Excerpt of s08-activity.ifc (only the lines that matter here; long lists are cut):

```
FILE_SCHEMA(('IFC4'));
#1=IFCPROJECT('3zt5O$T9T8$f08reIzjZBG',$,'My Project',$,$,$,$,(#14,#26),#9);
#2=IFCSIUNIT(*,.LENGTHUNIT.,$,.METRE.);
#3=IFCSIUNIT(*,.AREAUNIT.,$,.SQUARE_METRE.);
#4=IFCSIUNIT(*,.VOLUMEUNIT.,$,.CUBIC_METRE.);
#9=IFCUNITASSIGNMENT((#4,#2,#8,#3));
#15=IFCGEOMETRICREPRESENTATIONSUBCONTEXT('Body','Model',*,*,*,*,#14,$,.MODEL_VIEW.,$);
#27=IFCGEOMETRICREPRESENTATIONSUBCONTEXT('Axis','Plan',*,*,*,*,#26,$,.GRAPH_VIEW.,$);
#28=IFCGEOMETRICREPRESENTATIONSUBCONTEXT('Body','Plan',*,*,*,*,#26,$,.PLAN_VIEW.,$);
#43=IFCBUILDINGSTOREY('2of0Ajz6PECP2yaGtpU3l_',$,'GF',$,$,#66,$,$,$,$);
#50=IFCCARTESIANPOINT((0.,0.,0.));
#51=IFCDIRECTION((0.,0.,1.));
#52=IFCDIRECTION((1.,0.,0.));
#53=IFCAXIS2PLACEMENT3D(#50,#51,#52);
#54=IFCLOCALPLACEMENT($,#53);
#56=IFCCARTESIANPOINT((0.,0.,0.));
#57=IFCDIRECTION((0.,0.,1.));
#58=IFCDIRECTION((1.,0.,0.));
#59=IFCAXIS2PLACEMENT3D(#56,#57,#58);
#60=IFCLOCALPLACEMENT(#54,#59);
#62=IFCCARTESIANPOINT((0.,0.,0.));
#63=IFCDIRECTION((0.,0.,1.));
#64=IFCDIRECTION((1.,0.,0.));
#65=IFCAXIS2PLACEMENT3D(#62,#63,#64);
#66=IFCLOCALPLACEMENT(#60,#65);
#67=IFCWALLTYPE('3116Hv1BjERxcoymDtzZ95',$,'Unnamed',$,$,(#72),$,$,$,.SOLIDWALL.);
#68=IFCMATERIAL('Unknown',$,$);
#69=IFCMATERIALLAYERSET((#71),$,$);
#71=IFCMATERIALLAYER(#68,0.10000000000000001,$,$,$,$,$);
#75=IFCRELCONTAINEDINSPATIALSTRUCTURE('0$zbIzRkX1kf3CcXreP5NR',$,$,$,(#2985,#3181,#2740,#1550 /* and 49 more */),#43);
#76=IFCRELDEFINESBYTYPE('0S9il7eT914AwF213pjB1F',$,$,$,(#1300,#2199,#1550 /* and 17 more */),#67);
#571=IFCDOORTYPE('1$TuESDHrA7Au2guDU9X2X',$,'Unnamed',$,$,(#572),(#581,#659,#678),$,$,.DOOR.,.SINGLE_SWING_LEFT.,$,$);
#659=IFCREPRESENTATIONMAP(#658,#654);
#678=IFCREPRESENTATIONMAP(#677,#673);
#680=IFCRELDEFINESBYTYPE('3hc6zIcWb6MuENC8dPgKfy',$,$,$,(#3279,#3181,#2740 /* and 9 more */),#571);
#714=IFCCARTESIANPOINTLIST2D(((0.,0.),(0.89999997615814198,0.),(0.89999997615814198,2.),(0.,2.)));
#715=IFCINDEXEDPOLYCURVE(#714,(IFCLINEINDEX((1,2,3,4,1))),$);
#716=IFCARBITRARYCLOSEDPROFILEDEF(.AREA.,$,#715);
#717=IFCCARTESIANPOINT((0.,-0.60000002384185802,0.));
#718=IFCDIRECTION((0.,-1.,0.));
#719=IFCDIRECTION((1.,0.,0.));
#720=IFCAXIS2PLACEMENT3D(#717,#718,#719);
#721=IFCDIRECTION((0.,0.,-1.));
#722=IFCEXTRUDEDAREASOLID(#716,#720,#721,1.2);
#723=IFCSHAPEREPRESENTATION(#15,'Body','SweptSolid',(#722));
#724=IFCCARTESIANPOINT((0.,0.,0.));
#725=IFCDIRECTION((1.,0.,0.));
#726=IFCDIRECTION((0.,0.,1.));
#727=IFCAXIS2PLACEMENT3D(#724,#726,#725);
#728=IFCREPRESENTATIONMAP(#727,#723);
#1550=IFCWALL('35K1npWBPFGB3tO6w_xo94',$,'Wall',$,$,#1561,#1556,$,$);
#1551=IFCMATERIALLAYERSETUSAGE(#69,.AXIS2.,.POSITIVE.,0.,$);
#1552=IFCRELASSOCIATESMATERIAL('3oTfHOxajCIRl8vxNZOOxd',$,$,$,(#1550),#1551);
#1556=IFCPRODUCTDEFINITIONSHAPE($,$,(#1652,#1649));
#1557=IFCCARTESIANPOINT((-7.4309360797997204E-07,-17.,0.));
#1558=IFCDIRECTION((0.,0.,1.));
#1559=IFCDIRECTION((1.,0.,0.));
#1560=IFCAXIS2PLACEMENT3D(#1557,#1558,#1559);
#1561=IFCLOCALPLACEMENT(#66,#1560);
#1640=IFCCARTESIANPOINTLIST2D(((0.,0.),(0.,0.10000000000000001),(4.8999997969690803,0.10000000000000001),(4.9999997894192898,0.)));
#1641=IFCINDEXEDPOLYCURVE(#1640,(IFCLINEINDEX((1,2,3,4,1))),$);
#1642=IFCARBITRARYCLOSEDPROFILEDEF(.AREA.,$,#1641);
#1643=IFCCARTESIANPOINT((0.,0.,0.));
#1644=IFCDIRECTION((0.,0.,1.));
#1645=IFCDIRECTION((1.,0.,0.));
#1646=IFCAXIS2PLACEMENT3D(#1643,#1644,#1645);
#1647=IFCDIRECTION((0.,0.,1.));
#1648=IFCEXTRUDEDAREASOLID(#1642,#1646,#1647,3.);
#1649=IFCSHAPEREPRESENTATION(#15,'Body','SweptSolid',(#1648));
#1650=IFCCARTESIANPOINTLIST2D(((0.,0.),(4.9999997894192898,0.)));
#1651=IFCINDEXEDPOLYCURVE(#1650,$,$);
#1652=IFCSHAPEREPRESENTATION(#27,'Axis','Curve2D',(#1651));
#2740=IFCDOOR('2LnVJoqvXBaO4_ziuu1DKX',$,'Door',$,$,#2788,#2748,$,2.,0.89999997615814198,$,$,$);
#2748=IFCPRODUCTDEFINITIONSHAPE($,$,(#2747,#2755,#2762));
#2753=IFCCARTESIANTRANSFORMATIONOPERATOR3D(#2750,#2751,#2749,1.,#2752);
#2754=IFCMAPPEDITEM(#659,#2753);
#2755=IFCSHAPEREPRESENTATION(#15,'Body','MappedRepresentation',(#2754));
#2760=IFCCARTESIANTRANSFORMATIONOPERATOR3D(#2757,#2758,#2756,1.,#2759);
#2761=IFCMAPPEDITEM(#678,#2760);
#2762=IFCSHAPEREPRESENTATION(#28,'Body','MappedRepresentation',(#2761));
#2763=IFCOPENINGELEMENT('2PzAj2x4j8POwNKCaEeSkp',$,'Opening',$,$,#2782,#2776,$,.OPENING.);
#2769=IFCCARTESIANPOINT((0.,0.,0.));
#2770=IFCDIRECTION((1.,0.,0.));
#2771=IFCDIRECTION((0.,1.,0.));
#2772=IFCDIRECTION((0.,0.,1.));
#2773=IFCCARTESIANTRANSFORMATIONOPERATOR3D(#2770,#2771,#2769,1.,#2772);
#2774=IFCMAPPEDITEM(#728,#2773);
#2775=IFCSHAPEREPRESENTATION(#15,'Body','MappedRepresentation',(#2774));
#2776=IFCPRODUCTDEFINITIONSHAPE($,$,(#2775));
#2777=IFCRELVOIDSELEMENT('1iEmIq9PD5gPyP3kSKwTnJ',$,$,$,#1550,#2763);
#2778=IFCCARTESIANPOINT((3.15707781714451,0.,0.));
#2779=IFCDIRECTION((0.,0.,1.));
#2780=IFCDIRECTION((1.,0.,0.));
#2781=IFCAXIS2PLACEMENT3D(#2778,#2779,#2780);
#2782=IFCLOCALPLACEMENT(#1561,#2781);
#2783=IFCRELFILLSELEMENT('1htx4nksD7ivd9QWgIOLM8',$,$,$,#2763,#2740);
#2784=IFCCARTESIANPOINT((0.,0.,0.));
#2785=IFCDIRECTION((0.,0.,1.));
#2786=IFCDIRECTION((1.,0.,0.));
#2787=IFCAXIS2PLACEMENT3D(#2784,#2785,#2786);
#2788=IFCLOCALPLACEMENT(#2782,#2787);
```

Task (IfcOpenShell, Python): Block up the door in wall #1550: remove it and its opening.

```python
import ifcopenshell
import ifcopenshell.api.feature
import ifcopenshell.api.root
import ifcopenshell.geom
import ifcopenshell.util.shape

model = ifcopenshell.open("s08-activity.ifc")
settings = ifcopenshell.geom.settings()


def volume(element):
    """Net volume in cubic metres, openings subtracted."""
    shape = ifcopenshell.geom.create_shape(settings, element)
    return ifcopenshell.util.shape.get_volume(shape.geometry)


door = model.by_guid("2LnVJoqvXBaO4_ziuu1DKX")
opening = door.FillsVoids[0].RelatingOpeningElement
wall = opening.VoidsElements[0].RelatingBuildingElement
before = volume(wall)

ifcopenshell.api.root.remove_product(model, product=door)
ifcopenshell.api.feature.remove_feature(model, feature=opening)

after = volume(wall)

print(f"wall volume {before:.3f} -> {after:.3f} m3")

model.write("s08-activity_updated.ifc")
```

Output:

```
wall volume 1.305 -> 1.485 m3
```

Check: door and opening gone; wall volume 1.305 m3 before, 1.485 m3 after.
